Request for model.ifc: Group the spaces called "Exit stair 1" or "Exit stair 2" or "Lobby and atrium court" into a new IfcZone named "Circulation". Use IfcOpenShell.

First a look at what the model holds.

```python
import ifcopenshell

model = ifcopenshell.open("model.ifc")
print(model.schema)
seen = {}
for space in model.by_type("IfcSpace"):
    seen[space.LongName] = seen.get(space.LongName, 0) + 1
for name, count in sorted(seen.items(), key=str):
    print(count, "x", name)
print("zones:", [z.Name for z in model.by_type("IfcZone")][:20])
```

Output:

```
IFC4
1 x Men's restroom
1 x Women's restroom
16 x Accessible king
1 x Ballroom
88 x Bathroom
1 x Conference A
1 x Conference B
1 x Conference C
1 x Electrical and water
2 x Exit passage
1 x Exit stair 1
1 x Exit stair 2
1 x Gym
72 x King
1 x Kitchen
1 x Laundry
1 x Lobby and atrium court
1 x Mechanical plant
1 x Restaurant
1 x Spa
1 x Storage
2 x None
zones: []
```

```python
import ifcopenshell
import ifcopenshell.api.group
import ifcopenshell.api.root

model = ifcopenshell.open("model.ifc")

names = {"Exit stair 1", "Exit stair 2", "Lobby and atrium court"}
spaces = [s for s in model.by_type("IfcSpace") if s.LongName in names]

zone = ifcopenshell.api.root.create_entity(model, ifc_class="IfcZone", name="Circulation")
ifcopenshell.api.group.assign_group(model, products=spaces, group=zone)
print(len(spaces), "spaces in", zone.Name)

model.write("model_v2.ifc")
```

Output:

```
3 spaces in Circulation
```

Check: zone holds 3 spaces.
